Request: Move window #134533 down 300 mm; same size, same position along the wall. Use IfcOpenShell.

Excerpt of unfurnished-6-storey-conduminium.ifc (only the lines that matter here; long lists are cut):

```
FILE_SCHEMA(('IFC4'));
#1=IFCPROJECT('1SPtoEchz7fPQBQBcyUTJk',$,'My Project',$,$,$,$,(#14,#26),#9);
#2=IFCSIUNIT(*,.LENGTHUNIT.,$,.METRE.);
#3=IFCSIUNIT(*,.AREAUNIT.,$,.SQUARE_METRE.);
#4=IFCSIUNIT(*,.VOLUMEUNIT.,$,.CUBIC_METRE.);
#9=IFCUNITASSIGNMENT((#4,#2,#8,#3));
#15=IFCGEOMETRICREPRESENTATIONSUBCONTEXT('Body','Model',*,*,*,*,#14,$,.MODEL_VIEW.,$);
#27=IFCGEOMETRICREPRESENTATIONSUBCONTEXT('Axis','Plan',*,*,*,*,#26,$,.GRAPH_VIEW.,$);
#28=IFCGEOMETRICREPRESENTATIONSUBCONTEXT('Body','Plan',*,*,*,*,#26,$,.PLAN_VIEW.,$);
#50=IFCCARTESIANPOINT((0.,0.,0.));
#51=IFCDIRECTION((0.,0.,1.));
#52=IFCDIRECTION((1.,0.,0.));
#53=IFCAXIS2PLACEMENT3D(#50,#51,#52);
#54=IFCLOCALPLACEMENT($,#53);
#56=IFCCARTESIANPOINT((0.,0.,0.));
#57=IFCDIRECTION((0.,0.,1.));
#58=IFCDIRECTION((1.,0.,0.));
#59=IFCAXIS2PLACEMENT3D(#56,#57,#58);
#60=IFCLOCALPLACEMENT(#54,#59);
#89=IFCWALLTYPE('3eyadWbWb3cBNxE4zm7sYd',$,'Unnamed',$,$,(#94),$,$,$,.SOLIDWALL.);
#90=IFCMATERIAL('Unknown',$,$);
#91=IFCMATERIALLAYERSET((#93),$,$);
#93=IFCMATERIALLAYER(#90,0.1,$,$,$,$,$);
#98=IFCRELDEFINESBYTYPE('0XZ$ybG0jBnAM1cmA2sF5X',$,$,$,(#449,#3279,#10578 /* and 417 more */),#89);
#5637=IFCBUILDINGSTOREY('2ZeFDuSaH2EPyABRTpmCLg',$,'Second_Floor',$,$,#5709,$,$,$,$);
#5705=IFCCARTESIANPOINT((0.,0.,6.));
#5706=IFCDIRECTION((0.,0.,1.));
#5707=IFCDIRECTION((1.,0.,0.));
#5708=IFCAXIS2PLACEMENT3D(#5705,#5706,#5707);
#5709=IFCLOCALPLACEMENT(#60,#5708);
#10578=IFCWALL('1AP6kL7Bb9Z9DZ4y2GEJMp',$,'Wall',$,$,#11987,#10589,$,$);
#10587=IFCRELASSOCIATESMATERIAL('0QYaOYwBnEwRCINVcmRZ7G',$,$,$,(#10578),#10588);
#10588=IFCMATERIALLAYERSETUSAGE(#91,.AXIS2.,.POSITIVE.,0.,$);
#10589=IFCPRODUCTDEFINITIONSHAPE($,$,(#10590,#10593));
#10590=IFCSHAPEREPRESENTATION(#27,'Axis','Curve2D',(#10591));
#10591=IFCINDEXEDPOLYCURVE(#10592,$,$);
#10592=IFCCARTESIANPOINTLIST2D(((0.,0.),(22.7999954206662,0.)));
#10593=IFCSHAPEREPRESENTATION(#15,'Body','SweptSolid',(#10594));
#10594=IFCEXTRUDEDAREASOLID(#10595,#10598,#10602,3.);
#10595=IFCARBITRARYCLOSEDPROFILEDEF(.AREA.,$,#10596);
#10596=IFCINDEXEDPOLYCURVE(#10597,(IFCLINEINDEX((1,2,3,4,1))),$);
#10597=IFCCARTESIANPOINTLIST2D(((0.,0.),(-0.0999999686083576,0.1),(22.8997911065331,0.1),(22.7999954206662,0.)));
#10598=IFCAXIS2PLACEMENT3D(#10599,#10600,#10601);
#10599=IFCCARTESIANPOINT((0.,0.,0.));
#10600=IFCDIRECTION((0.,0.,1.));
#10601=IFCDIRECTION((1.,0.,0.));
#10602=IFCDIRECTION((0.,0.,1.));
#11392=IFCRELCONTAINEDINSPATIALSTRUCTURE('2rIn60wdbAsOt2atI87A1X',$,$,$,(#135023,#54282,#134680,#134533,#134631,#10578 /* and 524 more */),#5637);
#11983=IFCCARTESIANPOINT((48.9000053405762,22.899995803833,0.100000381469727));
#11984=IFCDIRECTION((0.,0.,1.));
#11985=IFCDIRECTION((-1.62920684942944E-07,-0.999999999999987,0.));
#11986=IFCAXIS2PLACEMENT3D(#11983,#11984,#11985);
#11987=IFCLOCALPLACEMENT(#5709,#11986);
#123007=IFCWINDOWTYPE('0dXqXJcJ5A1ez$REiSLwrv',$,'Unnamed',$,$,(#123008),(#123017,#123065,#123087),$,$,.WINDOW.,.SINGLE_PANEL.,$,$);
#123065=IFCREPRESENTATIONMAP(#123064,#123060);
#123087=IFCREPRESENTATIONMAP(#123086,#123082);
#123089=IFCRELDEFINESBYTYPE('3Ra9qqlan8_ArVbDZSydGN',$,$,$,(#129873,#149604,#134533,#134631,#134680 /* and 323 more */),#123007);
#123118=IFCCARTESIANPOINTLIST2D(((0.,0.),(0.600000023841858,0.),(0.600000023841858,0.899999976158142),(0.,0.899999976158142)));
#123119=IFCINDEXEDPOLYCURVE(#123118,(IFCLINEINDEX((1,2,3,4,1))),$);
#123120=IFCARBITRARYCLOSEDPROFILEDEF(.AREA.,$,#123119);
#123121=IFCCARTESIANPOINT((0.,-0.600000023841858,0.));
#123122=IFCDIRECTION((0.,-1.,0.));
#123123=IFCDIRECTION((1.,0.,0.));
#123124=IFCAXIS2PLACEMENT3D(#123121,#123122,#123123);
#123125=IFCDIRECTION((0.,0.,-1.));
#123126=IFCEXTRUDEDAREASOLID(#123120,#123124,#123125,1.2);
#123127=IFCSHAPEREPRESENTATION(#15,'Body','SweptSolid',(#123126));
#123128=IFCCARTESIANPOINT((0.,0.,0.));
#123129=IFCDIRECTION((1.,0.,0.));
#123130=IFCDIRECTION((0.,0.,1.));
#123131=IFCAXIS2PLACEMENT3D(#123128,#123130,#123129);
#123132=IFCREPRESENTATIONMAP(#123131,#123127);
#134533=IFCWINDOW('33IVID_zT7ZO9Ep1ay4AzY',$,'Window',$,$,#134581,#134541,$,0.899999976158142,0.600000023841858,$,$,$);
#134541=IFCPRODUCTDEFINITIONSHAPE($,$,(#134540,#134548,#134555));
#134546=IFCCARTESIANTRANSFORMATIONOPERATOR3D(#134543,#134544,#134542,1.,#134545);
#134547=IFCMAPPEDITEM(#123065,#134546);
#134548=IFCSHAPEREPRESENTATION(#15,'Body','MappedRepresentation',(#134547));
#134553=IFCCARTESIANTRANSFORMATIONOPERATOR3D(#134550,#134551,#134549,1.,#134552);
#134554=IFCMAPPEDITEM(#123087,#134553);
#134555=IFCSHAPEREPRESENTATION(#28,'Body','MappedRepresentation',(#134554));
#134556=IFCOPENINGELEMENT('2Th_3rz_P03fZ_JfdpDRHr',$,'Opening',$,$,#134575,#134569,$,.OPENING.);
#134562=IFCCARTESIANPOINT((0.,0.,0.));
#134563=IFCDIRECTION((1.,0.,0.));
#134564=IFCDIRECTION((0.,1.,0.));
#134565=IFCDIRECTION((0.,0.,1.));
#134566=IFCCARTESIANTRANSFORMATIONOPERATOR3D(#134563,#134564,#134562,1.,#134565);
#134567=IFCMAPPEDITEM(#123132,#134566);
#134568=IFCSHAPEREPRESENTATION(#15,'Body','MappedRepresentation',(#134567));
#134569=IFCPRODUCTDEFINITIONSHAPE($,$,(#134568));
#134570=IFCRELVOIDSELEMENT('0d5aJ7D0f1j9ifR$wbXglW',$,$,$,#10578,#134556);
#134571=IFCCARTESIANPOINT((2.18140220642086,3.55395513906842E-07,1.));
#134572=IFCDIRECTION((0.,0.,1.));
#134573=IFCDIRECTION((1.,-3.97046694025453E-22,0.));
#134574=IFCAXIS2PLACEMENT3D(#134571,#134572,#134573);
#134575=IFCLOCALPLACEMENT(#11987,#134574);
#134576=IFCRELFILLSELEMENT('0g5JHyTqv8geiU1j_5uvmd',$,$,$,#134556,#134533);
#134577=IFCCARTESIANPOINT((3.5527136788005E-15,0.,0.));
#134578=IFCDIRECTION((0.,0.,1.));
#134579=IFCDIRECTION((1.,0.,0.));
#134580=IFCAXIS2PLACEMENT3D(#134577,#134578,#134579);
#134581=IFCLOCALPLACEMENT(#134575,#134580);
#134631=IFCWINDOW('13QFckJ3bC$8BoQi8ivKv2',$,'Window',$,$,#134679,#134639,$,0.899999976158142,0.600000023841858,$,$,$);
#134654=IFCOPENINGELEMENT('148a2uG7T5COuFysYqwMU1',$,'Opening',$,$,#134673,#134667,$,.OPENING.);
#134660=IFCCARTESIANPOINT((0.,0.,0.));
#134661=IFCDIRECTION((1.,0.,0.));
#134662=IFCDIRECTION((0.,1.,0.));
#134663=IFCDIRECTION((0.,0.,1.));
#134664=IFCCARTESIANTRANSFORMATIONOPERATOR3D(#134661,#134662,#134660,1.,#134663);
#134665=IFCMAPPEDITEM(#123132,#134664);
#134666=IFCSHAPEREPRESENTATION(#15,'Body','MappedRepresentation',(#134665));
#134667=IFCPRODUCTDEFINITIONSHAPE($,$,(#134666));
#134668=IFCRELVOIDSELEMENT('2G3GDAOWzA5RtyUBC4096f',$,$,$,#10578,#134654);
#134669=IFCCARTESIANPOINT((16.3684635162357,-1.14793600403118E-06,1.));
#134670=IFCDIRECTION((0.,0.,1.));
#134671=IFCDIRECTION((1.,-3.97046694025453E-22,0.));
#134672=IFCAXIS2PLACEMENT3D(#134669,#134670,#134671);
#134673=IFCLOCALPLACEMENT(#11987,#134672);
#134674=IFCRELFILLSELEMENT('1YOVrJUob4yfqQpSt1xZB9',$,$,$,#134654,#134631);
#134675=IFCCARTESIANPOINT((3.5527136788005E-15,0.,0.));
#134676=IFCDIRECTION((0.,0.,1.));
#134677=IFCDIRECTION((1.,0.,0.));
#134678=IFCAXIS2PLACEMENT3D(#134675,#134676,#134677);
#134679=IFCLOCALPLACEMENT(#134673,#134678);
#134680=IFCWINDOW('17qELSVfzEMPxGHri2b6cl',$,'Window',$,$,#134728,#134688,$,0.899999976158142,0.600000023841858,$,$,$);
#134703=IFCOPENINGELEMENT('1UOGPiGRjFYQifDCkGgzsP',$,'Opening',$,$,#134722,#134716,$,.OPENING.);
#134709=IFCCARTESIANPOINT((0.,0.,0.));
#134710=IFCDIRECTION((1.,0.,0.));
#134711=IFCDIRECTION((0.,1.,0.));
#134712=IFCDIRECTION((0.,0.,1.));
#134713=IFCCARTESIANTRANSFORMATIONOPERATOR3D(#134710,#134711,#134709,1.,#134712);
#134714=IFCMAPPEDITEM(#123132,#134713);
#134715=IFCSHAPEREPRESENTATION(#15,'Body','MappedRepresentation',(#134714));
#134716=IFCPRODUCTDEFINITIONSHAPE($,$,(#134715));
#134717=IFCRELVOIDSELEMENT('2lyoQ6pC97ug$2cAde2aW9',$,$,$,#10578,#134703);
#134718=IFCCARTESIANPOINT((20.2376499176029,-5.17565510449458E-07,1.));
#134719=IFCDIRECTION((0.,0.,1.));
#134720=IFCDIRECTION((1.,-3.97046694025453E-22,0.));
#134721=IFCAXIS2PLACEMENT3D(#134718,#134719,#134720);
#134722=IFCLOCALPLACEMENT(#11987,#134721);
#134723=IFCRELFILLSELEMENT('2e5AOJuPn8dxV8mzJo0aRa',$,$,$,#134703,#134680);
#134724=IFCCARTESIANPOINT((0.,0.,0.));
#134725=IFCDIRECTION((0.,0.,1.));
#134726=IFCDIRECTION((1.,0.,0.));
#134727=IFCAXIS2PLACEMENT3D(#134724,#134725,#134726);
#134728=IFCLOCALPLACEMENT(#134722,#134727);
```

```python
import numpy as np
import ifcopenshell
import ifcopenshell.api.geometry
import ifcopenshell.util.placement
import ifcopenshell.util.unit

model = ifcopenshell.open("unfurnished-6-storey-conduminium.ifc")
unit_scale = ifcopenshell.util.unit.calculate_unit_scale(model)

window = model.by_guid("33IVID_zT7ZO9Ep1ay4AzY")
opening = window.FillsVoids[0].RelatingOpeningElement
dz = -0.3 / unit_scale

shift = np.array([0.0, 0.0, dz])
# The window is placed relative to its opening, so it follows when the opening moves.
matrix = ifcopenshell.util.placement.get_local_placement(opening.ObjectPlacement)
matrix[:3, 3] += shift
ifcopenshell.api.geometry.edit_object_placement(
    model, product=opening, matrix=matrix, is_si=False, should_transform_children=True
)

print(f"moved by {dz * unit_scale:+.3f} m")

model.write("unfurnished-6-storey-conduminium_rev.ifc")
```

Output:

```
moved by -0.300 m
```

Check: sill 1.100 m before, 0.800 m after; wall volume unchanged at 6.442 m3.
